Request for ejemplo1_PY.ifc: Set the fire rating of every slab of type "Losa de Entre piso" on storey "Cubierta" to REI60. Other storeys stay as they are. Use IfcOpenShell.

First a look at what the model holds.

```python
import ifcopenshell
import ifcopenshell.util.element

model = ifcopenshell.open("ejemplo1_PY.ifc")
print(model.schema)
storey = next(s for s in model.by_type("IfcBuildingStorey") if s.Name == "Cubierta")
slabs = [e for e in ifcopenshell.util.element.get_decomposition(storey) if e.is_a("IfcSlab")]
seen = {}
for e in slabs:
    element_type = ifcopenshell.util.element.get_type(e)
    key = (element_type.Name if element_type != e and element_type else None, ifcopenshell.util.element.get_pset(e, "Pset_SlabCommon", "FireRating"))
    seen[key] = seen.get(key, 0) + 1
for (name, value), count in sorted(seen.items(), key=str):
    print(count, "x", name, "|", value)
```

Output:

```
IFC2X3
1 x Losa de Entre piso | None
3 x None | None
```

```python
import ifcopenshell
import ifcopenshell.api.pset
import ifcopenshell.util.element

model = ifcopenshell.open("ejemplo1_PY.ifc")

storey = next(s for s in model.by_type("IfcBuildingStorey") if s.Name == "Cubierta")
slabs = [e for e in ifcopenshell.util.element.get_decomposition(storey) if e.is_a("IfcSlab")]

count = 0
for e in slabs:
    element_type = ifcopenshell.util.element.get_type(e)
    if element_type in (None, e) or element_type.Name != "Losa de Entre piso":
        continue
    # add_pset returns the element's existing set when there is one.
    pset = ifcopenshell.api.pset.add_pset(model, product=e, name="Pset_SlabCommon")
    ifcopenshell.api.pset.edit_pset(model, pset=pset, properties={"FireRating": "REI60"})
    count += 1

print(count, "slabs updated")

model.write("ejemplo1_PY-out.ifc")
```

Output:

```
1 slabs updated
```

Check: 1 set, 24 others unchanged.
